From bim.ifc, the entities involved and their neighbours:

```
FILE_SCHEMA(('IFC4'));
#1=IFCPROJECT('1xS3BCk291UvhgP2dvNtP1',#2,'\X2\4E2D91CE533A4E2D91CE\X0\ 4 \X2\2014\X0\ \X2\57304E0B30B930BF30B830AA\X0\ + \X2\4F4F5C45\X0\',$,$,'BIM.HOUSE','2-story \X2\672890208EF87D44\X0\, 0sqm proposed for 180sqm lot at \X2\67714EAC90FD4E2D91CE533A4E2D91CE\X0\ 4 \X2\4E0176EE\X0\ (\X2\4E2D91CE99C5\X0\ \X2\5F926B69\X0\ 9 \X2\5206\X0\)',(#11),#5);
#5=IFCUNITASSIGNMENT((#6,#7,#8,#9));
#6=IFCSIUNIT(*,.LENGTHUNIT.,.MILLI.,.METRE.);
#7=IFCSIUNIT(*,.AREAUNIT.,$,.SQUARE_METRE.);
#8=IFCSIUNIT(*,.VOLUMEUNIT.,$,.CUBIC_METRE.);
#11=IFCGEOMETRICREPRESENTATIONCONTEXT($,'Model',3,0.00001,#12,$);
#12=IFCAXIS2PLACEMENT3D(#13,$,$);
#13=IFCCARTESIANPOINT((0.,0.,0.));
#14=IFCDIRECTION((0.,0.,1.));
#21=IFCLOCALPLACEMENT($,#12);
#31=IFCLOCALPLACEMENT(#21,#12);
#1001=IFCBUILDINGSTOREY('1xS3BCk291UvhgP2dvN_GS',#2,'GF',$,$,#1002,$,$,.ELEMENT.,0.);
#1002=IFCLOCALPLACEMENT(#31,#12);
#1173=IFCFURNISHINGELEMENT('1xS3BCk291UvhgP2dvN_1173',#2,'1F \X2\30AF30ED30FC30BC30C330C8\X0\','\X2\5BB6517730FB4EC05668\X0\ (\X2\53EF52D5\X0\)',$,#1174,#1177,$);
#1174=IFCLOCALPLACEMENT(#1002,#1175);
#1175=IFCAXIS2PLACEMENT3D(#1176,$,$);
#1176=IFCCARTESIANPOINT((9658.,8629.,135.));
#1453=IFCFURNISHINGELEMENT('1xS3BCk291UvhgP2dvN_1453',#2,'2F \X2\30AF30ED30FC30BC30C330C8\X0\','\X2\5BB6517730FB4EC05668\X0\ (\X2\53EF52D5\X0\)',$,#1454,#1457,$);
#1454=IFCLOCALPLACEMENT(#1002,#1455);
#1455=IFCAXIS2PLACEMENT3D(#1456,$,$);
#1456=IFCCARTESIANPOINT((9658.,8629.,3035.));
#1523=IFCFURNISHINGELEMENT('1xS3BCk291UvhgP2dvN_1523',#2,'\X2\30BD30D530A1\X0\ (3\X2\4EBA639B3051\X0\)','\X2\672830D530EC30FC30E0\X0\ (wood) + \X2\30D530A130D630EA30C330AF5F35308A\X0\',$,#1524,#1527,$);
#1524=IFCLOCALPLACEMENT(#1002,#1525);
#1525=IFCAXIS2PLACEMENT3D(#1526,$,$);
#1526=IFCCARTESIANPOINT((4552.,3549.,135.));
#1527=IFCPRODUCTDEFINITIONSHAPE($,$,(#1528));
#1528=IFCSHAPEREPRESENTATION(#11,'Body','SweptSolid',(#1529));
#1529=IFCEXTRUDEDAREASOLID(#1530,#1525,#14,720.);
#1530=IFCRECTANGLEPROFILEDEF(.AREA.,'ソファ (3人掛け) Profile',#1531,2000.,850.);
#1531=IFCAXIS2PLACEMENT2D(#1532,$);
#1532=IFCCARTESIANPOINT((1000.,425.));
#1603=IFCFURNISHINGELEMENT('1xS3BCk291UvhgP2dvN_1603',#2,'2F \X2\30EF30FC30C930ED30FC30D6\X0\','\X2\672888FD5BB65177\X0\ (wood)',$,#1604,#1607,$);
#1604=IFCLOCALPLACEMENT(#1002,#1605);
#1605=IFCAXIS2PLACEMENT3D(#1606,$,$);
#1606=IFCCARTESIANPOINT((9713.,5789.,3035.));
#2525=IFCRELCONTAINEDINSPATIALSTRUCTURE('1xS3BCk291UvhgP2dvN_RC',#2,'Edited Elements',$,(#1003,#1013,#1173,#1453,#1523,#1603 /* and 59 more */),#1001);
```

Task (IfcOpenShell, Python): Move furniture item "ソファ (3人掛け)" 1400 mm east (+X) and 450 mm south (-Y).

```python
import ifcopenshell
import ifcopenshell.api.geometry
import ifcopenshell.util.placement
import ifcopenshell.util.unit

model = ifcopenshell.open("bim.ifc")
unit_scale = ifcopenshell.util.unit.calculate_unit_scale(model)

item = model.by_guid("1xS3BCk291UvhgP2dvN_1523")
matrix = ifcopenshell.util.placement.get_local_placement(item.ObjectPlacement)
matrix[0, 3] += 1.4 / unit_scale
matrix[1, 3] -= 0.45 / unit_scale
ifcopenshell.api.geometry.edit_object_placement(model, product=item, matrix=matrix, is_si=False)

print(ifcopenshell.util.placement.get_local_placement(item.ObjectPlacement).round(3) + 0.0)

model.write("bim-out.ifc")
```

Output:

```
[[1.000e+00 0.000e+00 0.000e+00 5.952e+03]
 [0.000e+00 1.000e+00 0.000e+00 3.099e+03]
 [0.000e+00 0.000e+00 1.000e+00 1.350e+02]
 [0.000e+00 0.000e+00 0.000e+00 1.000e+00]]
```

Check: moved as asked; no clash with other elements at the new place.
